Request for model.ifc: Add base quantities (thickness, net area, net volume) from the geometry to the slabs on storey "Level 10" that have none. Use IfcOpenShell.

First a look at what the model holds.

```python
import ifcopenshell
import ifcopenshell.util.element
import ifcopenshell.util.unit

model = ifcopenshell.open("model.ifc")
print(model.schema)
for unit_type in ("LENGTHUNIT", "AREAUNIT", "VOLUMEUNIT"):
    print(unit_type, ifcopenshell.util.unit.calculate_unit_scale(model, unit_type))
storey = next(s for s in model.by_type("IfcBuildingStorey") if s.Name == "Level 10")
slabs = [e for e in ifcopenshell.util.element.get_decomposition(storey) if e.is_a("IfcSlab")]
for e in sorted(slabs, key=lambda e: e.id()):
    print(e.id(), e.is_a(), e.Name, list(ifcopenshell.util.element.get_psets(e, qtos_only=True)), sep=" | ")
```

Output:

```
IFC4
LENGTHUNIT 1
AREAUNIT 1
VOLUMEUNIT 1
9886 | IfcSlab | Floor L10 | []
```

```python
import ifcopenshell
import ifcopenshell.api.pset
import ifcopenshell.geom
import ifcopenshell.util.element
import ifcopenshell.util.shape
import ifcopenshell.util.unit

model = ifcopenshell.open("model.ifc")
unit_scale = ifcopenshell.util.unit.calculate_unit_scale(model)
area_scale = ifcopenshell.util.unit.calculate_unit_scale(model, "AREAUNIT")
volume_scale = ifcopenshell.util.unit.calculate_unit_scale(model, "VOLUMEUNIT")
settings = ifcopenshell.geom.settings()

storey = next(s for s in model.by_type("IfcBuildingStorey") if s.Name == "Level 10")
slabs = [e for e in ifcopenshell.util.element.get_decomposition(storey) if e.is_a("IfcSlab")]

for e in sorted(slabs, key=lambda e: e.id()):
    if ifcopenshell.util.element.get_psets(e, qtos_only=True, should_inherit=False):
        continue
    # Geometry comes back in metres, in the element's own axes.
    shape = ifcopenshell.geom.create_shape(settings, e)
    values = {
        "Width": ifcopenshell.util.shape.get_z(shape.geometry) / unit_scale,
        "NetArea": ifcopenshell.util.shape.get_footprint_area(shape.geometry) / area_scale,
        "NetVolume": ifcopenshell.util.shape.get_volume(shape.geometry) / volume_scale,
    }
    qto = ifcopenshell.api.pset.add_qto(model, product=e, name="Qto_SlabBaseQuantities")
    ifcopenshell.api.pset.edit_qto(model, qto=qto, properties=values)
    print(e.id(), {k: round(v, 3) for k, v in values.items()})

model.write("model_rev.ifc")
```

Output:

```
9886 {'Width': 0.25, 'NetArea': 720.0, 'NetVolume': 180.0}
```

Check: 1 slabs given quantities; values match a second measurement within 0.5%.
